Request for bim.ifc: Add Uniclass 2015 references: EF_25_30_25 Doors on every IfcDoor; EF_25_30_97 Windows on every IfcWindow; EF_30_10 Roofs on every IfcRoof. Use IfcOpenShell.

First a look at what the model holds.

```python
import ifcopenshell

model = ifcopenshell.open("bim.ifc")
print(model.schema)
print("classifications:", [c.Name for c in model.by_type("IfcClassification")])
for ifc_class in ("IfcDoor", "IfcRoof", "IfcStair", "IfcWall", "IfcWindow"):
    print(ifc_class, len(model.by_type(ifc_class)))
```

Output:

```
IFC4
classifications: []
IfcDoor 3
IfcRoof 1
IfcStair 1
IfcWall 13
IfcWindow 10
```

```python
import ifcopenshell
import ifcopenshell.api.classification

model = ifcopenshell.open("bim.ifc")

system = ifcopenshell.api.classification.add_classification(model, classification="Uniclass 2015")

codes = {
    "IfcDoor": ("EF_25_30_25", "Doors"),
    "IfcWindow": ("EF_25_30_97", "Windows"),
    "IfcRoof": ("EF_30_10", "Roofs"),
}
for ifc_class, (code, name) in codes.items():
    products = model.by_type(ifc_class)
    ifcopenshell.api.classification.add_reference(
        model, products=products, classification=system, identification=code, name=name
    )
    print(code, len(products))

model.write("bim_updated.ifc")
```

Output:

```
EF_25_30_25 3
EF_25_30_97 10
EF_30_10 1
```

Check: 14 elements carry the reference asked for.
